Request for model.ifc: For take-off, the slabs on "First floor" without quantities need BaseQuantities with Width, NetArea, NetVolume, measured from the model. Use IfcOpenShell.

First a look at what the model holds.

```python
import ifcopenshell
import ifcopenshell.util.element
import ifcopenshell.util.unit

model = ifcopenshell.open("model.ifc")
print(model.schema)
for unit_type in ("LENGTHUNIT", "AREAUNIT", "VOLUMEUNIT"):
    print(unit_type, ifcopenshell.util.unit.calculate_unit_scale(model, unit_type))
storey = next(s for s in model.by_type("IfcBuildingStorey") if s.Name == "First floor")
slabs = [e for e in ifcopenshell.util.element.get_decomposition(storey) if e.is_a("IfcSlab")]
for e in sorted(slabs, key=lambda e: e.id()):
    print(e.id(), e.is_a(), e.Name, list(ifcopenshell.util.element.get_psets(e, qtos_only=True)), sep=" | ")
```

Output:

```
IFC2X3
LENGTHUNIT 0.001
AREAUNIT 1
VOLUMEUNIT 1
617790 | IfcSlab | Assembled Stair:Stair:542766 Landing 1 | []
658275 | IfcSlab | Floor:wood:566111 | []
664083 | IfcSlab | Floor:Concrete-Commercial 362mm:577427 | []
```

```python
import ifcopenshell
import ifcopenshell.api.pset
import ifcopenshell.geom
import ifcopenshell.util.element
import ifcopenshell.util.shape
import ifcopenshell.util.unit

model = ifcopenshell.open("model.ifc")
unit_scale = ifcopenshell.util.unit.calculate_unit_scale(model)
area_scale = ifcopenshell.util.unit.calculate_unit_scale(model, "AREAUNIT")
volume_scale = ifcopenshell.util.unit.calculate_unit_scale(model, "VOLUMEUNIT")
settings = ifcopenshell.geom.settings()

storey = next(s for s in model.by_type("IfcBuildingStorey") if s.Name == "First floor")
slabs = [e for e in ifcopenshell.util.element.get_decomposition(storey) if e.is_a("IfcSlab")]

for e in sorted(slabs, key=lambda e: e.id()):
    if ifcopenshell.util.element.get_psets(e, qtos_only=True, should_inherit=False):
        continue
    # Geometry comes back in metres, in the element's own axes.
    shape = ifcopenshell.geom.create_shape(settings, e)
    values = {
        "Width": ifcopenshell.util.shape.get_z(shape.geometry) / unit_scale,
        "NetArea": ifcopenshell.util.shape.get_footprint_area(shape.geometry) / area_scale,
        "NetVolume": ifcopenshell.util.shape.get_volume(shape.geometry) / volume_scale,
    }
    qto = ifcopenshell.api.pset.add_qto(model, product=e, name="BaseQuantities")
    ifcopenshell.api.pset.edit_qto(model, qto=qto, properties=values)
    print(e.id(), {k: round(v, 3) for k, v in values.items()})

model.write("model_rev.ifc")
```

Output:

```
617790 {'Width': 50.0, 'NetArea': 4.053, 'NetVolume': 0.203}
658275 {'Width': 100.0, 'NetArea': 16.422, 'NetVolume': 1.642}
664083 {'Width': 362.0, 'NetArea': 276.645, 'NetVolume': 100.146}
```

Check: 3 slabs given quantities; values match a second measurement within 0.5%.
